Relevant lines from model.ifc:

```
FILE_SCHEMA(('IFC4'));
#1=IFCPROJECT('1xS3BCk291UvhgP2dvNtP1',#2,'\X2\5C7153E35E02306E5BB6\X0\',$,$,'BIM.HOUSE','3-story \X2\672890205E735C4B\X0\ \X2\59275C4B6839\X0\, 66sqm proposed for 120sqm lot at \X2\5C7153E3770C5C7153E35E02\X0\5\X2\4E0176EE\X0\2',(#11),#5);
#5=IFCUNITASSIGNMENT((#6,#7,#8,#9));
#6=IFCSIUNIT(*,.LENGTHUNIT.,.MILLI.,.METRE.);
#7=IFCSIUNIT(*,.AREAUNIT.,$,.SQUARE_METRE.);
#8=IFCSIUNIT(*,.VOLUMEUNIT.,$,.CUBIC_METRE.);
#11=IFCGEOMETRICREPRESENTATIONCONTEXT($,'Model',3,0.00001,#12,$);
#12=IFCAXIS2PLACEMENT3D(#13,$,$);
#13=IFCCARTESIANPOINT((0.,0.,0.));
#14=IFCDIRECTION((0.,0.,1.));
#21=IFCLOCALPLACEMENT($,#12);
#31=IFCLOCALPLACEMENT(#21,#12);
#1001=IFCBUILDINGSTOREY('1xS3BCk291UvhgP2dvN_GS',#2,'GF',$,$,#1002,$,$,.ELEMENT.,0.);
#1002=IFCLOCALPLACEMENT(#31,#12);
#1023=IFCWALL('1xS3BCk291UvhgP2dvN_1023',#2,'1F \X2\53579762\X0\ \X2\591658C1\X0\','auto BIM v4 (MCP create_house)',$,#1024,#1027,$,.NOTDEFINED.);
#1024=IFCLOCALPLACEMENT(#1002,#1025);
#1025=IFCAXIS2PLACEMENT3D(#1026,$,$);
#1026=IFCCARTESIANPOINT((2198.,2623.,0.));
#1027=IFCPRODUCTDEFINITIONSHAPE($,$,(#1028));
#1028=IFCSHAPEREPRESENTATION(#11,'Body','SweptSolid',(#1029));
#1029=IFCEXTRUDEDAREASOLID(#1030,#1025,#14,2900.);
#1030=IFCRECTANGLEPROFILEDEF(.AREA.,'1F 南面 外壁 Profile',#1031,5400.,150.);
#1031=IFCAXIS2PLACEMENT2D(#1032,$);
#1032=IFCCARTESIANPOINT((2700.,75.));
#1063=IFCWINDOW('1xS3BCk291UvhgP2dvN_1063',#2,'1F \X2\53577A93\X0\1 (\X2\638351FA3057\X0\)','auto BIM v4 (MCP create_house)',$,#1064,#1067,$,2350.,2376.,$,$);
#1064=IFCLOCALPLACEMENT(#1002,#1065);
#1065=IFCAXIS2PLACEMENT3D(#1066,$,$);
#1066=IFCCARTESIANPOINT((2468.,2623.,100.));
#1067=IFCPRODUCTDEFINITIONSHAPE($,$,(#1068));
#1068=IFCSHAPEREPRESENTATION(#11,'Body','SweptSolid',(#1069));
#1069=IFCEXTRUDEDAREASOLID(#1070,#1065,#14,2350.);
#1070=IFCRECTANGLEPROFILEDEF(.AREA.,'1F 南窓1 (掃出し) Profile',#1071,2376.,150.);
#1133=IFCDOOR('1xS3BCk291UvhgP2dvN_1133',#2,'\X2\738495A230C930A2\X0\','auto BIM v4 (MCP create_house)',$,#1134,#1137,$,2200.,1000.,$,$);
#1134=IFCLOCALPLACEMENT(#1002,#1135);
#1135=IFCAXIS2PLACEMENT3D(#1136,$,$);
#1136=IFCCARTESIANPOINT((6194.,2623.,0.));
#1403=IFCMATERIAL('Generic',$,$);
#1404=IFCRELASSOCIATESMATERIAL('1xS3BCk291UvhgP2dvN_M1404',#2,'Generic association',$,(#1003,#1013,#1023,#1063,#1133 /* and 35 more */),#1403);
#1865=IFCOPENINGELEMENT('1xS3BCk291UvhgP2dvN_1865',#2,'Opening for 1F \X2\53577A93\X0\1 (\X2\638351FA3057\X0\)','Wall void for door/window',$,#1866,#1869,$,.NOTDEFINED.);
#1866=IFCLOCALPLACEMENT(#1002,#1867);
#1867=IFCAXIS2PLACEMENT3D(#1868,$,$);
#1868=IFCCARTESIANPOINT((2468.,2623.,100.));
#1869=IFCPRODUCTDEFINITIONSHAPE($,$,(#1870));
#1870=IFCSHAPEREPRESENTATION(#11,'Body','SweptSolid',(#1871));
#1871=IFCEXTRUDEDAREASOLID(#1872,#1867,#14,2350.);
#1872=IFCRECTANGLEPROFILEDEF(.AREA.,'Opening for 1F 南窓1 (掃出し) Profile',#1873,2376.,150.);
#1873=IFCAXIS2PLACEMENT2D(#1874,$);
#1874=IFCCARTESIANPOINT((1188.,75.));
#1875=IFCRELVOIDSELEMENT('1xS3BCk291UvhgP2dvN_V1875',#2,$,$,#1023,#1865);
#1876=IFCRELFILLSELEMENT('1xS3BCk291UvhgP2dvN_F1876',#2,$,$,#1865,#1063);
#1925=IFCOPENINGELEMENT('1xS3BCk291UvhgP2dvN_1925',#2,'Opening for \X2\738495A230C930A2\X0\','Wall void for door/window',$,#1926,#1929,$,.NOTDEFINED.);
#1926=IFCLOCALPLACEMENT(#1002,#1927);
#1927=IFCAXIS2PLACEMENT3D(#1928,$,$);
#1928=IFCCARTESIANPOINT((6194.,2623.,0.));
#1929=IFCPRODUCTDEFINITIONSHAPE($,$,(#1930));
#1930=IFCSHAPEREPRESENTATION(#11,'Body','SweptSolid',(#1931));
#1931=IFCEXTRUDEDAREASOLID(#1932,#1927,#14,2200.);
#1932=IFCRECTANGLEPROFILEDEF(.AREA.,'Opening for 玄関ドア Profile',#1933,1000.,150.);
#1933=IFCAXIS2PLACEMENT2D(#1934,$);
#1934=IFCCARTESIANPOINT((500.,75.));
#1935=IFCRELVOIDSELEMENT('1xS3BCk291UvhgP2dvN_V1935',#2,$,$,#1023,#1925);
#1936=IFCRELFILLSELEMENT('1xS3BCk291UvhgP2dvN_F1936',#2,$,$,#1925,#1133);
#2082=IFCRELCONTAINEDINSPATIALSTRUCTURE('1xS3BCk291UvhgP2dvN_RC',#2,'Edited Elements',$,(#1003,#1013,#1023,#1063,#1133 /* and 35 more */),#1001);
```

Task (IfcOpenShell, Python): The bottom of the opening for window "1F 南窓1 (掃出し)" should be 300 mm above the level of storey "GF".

```python
import numpy as np
import ifcopenshell
import ifcopenshell.api.geometry
import ifcopenshell.geom
import ifcopenshell.util.element
import ifcopenshell.util.placement
import ifcopenshell.util.shape
import ifcopenshell.util.unit

model = ifcopenshell.open("model.ifc")
unit_scale = ifcopenshell.util.unit.calculate_unit_scale(model)

window = model.by_id(1063)
opening = window.FillsVoids[0].RelatingOpeningElement
storey = ifcopenshell.util.element.get_container(window, ifc_class="IfcBuildingStorey")
level = ifcopenshell.util.placement.get_local_placement(storey.ObjectPlacement)[2, 3]

# The opening's origin need not be at the sill, so measure its lowest point.
shape = ifcopenshell.geom.create_shape(ifcopenshell.geom.settings(), opening)
bottom = ifcopenshell.util.shape.get_shape_bottom_elevation(shape, shape.geometry) / unit_scale
dz = level + 0.3 / unit_scale - bottom

shift = np.array([0.0, 0.0, dz])
# The window is not placed relative to its opening, so move both.
for product in (opening, window):
    matrix = ifcopenshell.util.placement.get_local_placement(product.ObjectPlacement)
    matrix[:3, 3] += shift
    ifcopenshell.api.geometry.edit_object_placement(model, product=product, matrix=matrix, is_si=False)

print(f"moved by {dz * unit_scale:+.3f} m")

model.write("model_v2.ifc")
```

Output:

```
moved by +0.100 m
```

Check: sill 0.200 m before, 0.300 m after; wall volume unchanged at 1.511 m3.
